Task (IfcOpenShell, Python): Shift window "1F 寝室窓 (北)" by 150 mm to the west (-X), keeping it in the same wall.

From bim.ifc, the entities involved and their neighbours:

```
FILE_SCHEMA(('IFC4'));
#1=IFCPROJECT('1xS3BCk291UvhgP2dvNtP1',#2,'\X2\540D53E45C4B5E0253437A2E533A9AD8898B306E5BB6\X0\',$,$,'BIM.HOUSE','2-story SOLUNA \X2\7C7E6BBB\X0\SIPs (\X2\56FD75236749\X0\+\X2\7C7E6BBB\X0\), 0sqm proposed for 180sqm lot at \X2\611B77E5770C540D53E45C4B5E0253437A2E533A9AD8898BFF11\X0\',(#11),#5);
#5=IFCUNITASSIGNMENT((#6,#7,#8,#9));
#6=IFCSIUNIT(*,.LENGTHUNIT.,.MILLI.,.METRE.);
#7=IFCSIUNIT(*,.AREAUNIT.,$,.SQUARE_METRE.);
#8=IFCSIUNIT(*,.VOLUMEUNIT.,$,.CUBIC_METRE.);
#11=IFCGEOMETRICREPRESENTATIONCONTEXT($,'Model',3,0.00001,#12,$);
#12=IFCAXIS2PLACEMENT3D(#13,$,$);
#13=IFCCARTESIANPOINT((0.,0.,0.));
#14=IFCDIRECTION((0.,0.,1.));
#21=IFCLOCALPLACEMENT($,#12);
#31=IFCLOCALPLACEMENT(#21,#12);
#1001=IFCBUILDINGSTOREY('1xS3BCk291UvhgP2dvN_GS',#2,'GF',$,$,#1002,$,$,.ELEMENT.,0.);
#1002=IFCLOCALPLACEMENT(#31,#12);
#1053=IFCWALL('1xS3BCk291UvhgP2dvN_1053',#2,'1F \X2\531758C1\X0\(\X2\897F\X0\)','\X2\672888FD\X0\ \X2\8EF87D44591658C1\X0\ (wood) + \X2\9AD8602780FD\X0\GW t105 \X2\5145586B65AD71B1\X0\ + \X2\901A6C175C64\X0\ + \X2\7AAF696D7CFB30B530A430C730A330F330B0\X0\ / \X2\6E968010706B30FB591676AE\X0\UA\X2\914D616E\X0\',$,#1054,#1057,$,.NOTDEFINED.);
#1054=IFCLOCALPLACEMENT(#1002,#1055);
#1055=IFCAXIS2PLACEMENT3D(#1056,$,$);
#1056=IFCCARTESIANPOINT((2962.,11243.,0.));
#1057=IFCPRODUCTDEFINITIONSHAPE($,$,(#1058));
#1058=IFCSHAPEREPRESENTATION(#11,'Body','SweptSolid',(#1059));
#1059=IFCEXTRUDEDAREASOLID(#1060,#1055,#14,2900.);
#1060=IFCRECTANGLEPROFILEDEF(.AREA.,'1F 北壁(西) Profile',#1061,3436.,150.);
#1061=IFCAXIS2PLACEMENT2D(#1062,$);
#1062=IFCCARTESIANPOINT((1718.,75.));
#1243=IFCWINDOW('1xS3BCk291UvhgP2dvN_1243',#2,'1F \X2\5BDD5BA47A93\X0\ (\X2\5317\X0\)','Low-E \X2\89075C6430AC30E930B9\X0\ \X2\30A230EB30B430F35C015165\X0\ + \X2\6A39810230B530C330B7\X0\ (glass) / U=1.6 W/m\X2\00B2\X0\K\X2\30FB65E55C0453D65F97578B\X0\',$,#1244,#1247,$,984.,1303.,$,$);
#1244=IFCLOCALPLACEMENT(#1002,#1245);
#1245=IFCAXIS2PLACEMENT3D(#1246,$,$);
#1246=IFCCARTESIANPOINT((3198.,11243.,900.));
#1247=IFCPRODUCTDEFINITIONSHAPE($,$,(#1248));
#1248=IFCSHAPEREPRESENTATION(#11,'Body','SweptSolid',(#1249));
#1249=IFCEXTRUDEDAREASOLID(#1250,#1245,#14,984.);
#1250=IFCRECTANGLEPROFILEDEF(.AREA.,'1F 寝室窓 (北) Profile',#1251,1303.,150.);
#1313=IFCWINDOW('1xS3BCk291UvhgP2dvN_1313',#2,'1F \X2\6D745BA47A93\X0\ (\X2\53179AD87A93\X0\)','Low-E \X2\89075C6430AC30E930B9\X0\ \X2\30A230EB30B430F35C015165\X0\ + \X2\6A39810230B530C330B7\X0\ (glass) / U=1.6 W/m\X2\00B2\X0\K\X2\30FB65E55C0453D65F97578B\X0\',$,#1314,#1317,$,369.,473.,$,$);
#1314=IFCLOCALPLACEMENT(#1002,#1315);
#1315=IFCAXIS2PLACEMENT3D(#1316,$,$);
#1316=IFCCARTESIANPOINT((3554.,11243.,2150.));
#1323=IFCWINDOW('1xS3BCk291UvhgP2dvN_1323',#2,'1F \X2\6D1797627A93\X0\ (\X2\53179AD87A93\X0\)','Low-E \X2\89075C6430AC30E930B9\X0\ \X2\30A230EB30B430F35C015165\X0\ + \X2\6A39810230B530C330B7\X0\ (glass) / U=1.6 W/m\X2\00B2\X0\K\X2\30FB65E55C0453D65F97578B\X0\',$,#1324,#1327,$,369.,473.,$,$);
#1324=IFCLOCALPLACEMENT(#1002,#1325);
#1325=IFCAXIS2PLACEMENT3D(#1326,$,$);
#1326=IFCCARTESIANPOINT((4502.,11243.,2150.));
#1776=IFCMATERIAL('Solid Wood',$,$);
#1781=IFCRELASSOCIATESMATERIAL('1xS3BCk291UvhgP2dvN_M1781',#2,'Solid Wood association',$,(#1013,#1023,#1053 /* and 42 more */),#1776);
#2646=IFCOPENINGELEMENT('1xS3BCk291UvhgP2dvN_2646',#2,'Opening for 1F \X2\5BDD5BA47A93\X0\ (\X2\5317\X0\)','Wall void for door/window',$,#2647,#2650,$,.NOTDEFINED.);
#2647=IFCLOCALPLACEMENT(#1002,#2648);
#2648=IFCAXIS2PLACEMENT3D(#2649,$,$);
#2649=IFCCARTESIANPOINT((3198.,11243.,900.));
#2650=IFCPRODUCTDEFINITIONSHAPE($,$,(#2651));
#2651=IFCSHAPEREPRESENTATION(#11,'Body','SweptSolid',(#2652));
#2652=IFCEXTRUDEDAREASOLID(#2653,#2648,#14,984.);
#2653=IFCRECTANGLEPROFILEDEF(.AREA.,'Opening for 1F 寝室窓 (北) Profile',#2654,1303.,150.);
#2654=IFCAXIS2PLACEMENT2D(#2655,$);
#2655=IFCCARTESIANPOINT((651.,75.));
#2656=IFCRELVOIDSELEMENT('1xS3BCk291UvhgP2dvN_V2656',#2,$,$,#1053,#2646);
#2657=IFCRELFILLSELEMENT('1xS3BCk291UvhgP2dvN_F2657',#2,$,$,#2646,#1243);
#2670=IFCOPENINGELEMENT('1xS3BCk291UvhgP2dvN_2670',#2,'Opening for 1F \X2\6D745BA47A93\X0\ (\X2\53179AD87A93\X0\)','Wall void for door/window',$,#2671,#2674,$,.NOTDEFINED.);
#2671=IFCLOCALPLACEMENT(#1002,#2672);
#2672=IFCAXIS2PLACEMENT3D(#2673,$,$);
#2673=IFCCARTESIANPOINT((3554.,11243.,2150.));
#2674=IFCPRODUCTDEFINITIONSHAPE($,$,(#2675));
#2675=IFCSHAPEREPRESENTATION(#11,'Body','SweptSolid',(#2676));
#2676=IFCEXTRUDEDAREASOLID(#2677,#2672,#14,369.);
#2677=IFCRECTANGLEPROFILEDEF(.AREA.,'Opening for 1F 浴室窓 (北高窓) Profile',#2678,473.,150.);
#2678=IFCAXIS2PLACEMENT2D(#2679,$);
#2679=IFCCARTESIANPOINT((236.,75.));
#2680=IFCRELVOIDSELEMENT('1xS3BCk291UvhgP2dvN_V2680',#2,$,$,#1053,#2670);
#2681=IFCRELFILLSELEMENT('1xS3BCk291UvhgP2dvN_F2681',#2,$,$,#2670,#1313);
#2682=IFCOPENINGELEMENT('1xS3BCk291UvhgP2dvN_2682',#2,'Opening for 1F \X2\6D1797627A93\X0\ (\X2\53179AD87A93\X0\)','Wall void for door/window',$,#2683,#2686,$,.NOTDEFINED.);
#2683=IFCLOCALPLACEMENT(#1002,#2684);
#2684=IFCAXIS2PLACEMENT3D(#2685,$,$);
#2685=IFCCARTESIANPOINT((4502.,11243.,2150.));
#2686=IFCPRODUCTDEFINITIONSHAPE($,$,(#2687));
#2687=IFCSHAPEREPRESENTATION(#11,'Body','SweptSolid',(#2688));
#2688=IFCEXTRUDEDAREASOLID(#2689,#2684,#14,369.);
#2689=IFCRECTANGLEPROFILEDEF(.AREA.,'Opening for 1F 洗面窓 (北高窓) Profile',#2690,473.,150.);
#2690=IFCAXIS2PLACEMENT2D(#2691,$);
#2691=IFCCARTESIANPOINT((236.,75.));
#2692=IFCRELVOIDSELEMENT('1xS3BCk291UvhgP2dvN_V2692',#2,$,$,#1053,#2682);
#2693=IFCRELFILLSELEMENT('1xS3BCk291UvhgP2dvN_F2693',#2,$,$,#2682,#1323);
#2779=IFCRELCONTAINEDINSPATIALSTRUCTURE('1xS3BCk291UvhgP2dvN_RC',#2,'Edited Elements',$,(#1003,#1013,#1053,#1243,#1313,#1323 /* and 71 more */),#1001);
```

```python
import ifcopenshell
import ifcopenshell.api.geometry
import ifcopenshell.util.placement
import ifcopenshell.util.unit

model = ifcopenshell.open("bim.ifc")
unit_scale = ifcopenshell.util.unit.calculate_unit_scale(model)

window = model.by_id(1243)
opening = window.FillsVoids[0].RelatingOpeningElement
wall = opening.VoidsElements[0].RelatingBuildingElement

wall_matrix = ifcopenshell.util.placement.get_local_placement(wall.ObjectPlacement)
shift = wall_matrix[:3, 0] * -0.15 / unit_scale
before = ifcopenshell.util.placement.get_local_placement(window.ObjectPlacement)[:3, 3].copy()

# The window is not placed relative to its opening, so move both.
for product in (opening, window):
    matrix = ifcopenshell.util.placement.get_local_placement(product.ObjectPlacement)
    matrix[:3, 3] += shift
    ifcopenshell.api.geometry.edit_object_placement(model, product=product, matrix=matrix, is_si=False)

after = ifcopenshell.util.placement.get_local_placement(window.ObjectPlacement)[:3, 3]
print("window moved by", (after - before).round(3) + 0.0)

model.write("bim_updated.ifc")
```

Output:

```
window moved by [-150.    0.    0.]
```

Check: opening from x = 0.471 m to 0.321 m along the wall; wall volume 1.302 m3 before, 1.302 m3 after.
